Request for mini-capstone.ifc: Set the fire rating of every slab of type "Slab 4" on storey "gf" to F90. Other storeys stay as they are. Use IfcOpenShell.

First a look at what the model holds.

```python
import ifcopenshell
import ifcopenshell.util.element

model = ifcopenshell.open("mini-capstone.ifc")
print(model.schema)
storey = next(s for s in model.by_type("IfcBuildingStorey") if s.Name == "gf")
slabs = [e for e in ifcopenshell.util.element.get_decomposition(storey) if e.is_a("IfcSlab")]
seen = {}
for e in slabs:
    element_type = ifcopenshell.util.element.get_type(e)
    key = (element_type.Name if element_type != e and element_type else None, ifcopenshell.util.element.get_pset(e, "Pset_SlabCommon", "FireRating"))
    seen[key] = seen.get(key, 0) + 1
for (name, value), count in sorted(seen.items(), key=str):
    print(count, "x", name, "|", value)
```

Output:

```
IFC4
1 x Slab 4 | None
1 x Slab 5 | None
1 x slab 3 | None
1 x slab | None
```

```python
import ifcopenshell
import ifcopenshell.api.pset
import ifcopenshell.util.element

model = ifcopenshell.open("mini-capstone.ifc")

storey = next(s for s in model.by_type("IfcBuildingStorey") if s.Name == "gf")
slabs = [e for e in ifcopenshell.util.element.get_decomposition(storey) if e.is_a("IfcSlab")]

count = 0
for e in slabs:
    element_type = ifcopenshell.util.element.get_type(e)
    if element_type in (None, e) or element_type.Name != "Slab 4":
        continue
    # add_pset returns the element's existing set when there is one.
    pset = ifcopenshell.api.pset.add_pset(model, product=e, name="Pset_SlabCommon")
    ifcopenshell.api.pset.edit_pset(model, pset=pset, properties={"FireRating": "F90"})
    count += 1

print(count, "slabs updated")

model.write("mini-capstone-out.ifc")
```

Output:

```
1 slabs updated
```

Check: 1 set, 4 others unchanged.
